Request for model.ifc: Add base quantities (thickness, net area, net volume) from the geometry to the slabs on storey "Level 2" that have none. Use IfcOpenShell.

First a look at what the model holds.

```python
import ifcopenshell
import ifcopenshell.util.element
import ifcopenshell.util.unit

model = ifcopenshell.open("model.ifc")
print(model.schema)
for unit_type in ("LENGTHUNIT", "AREAUNIT", "VOLUMEUNIT"):
    print(unit_type, ifcopenshell.util.unit.calculate_unit_scale(model, unit_type))
storey = next(s for s in model.by_type("IfcBuildingStorey") if s.Name == "Level 2")
slabs = [e for e in ifcopenshell.util.element.get_decomposition(storey) if e.is_a("IfcSlab")]
for e in sorted(slabs, key=lambda e: e.id()):
    print(e.id(), e.is_a(), e.Name, list(ifcopenshell.util.element.get_psets(e, qtos_only=True)), sep=" | ")
```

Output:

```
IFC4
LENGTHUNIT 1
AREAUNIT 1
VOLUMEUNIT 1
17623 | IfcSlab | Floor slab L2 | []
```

```python
import ifcopenshell
import ifcopenshell.api.pset
import ifcopenshell.geom
import ifcopenshell.util.element
import ifcopenshell.util.shape
import ifcopenshell.util.unit

model = ifcopenshell.open("model.ifc")
unit_scale = ifcopenshell.util.unit.calculate_unit_scale(model)
area_scale = ifcopenshell.util.unit.calculate_unit_scale(model, "AREAUNIT")
volume_scale = ifcopenshell.util.unit.calculate_unit_scale(model, "VOLUMEUNIT")
settings = ifcopenshell.geom.settings()

storey = next(s for s in model.by_type("IfcBuildingStorey") if s.Name == "Level 2")
slabs = [e for e in ifcopenshell.util.element.get_decomposition(storey) if e.is_a("IfcSlab")]

for e in sorted(slabs, key=lambda e: e.id()):
    if ifcopenshell.util.element.get_psets(e, qtos_only=True, should_inherit=False):
        continue
    # Geometry comes back in metres, in the element's own axes.
    shape = ifcopenshell.geom.create_shape(settings, e)
    values = {
        "Width": ifcopenshell.util.shape.get_z(shape.geometry) / unit_scale,
        "NetArea": ifcopenshell.util.shape.get_footprint_area(shape.geometry) / area_scale,
        "NetVolume": ifcopenshell.util.shape.get_volume(shape.geometry) / volume_scale,
    }
    qto = ifcopenshell.api.pset.add_qto(model, product=e, name="Qto_SlabBaseQuantities")
    ifcopenshell.api.pset.edit_qto(model, qto=qto, properties=values)
    print(e.id(), {k: round(v, 3) for k, v in values.items()})

model.write("model_edited.ifc")
```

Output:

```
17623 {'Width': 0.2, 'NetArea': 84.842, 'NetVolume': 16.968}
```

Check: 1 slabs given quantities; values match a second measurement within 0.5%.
